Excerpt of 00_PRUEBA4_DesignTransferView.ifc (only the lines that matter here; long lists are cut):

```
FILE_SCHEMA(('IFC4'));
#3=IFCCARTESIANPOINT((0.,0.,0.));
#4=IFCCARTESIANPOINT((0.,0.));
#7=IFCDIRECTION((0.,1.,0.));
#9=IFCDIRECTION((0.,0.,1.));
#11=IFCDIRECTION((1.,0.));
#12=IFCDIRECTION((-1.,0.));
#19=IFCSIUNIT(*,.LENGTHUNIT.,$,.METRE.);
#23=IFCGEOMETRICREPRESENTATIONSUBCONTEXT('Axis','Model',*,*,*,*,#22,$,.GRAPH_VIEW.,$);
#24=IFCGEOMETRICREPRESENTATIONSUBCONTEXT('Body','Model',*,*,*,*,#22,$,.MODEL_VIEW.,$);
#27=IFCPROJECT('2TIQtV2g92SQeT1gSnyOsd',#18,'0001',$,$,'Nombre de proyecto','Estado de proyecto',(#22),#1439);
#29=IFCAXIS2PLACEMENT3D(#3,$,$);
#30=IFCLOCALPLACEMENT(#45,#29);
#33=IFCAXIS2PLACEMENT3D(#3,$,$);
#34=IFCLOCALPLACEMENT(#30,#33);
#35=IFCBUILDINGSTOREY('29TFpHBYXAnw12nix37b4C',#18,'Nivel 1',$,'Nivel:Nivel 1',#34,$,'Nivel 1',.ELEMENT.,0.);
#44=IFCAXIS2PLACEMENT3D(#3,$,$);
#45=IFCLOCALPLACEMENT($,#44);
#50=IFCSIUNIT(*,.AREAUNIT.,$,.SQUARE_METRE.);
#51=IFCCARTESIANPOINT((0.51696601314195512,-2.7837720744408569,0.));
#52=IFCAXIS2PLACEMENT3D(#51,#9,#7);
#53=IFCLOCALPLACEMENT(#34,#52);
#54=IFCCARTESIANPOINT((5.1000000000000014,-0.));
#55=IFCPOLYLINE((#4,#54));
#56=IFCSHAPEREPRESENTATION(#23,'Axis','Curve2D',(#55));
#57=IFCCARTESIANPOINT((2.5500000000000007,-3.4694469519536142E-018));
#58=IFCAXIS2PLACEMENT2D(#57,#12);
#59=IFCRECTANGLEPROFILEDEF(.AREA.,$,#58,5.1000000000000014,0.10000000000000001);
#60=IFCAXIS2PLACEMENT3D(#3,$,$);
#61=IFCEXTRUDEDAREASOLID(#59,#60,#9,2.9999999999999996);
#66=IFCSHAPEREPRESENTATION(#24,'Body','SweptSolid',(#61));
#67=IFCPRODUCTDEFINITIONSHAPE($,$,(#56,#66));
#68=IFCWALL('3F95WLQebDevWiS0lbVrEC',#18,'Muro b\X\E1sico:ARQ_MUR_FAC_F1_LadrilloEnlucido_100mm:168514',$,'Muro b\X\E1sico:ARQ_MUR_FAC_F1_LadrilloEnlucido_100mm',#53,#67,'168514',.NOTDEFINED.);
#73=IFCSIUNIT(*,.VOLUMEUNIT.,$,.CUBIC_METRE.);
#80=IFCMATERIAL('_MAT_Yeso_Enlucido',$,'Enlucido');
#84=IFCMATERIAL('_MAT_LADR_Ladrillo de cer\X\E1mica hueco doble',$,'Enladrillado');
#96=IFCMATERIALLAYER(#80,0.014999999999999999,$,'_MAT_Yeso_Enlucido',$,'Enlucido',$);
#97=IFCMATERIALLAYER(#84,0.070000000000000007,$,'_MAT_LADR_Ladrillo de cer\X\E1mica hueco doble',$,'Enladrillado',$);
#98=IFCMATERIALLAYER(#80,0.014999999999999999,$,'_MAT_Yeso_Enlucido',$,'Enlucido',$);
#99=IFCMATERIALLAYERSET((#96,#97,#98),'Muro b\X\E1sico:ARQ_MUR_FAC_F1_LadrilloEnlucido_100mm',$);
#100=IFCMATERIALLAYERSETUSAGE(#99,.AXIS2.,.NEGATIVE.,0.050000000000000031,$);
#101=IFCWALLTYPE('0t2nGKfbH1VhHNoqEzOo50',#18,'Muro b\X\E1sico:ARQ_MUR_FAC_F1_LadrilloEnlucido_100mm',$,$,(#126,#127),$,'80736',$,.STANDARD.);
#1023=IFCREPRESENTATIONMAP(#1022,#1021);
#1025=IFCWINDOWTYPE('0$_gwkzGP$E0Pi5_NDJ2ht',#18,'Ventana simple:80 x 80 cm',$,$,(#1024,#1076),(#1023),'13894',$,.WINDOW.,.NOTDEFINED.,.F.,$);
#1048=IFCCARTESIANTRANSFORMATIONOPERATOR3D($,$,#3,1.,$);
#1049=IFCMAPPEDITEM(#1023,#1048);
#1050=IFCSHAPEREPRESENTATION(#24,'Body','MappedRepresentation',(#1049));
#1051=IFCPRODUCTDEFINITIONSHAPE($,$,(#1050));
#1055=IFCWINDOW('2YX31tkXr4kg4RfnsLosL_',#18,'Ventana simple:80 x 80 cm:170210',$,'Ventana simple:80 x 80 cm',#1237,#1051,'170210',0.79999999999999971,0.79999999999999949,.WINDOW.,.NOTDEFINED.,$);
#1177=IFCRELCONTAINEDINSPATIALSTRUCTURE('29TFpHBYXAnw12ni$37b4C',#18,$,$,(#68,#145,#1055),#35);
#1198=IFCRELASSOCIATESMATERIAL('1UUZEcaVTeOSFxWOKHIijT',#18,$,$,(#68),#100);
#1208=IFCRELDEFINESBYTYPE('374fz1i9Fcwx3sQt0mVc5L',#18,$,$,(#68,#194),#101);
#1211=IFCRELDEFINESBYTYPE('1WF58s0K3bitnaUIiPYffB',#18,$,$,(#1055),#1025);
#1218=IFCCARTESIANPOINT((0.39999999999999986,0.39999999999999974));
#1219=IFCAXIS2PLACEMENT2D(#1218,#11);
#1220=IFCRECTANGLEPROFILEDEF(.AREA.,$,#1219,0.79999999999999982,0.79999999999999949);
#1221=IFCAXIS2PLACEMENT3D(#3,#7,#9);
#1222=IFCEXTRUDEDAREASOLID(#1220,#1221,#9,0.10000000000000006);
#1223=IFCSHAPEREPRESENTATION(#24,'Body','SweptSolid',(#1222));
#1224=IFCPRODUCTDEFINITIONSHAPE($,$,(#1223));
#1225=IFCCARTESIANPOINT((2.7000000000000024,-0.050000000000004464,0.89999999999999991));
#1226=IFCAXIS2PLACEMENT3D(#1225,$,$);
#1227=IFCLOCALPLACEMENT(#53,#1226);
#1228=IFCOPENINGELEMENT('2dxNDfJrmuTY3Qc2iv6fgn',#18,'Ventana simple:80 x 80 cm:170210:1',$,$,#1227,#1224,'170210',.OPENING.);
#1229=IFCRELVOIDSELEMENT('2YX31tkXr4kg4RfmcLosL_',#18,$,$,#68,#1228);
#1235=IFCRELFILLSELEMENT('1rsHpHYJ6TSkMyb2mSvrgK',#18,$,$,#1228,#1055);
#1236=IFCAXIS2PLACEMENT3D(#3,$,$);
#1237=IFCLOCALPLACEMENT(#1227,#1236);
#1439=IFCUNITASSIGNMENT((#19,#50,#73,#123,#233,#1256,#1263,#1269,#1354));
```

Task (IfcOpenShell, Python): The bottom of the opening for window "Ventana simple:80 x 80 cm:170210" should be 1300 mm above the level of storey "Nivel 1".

```python
import numpy as np
import ifcopenshell
import ifcopenshell.api.geometry
import ifcopenshell.geom
import ifcopenshell.util.element
import ifcopenshell.util.placement
import ifcopenshell.util.shape
import ifcopenshell.util.unit

model = ifcopenshell.open("00_PRUEBA4_DesignTransferView.ifc")
unit_scale = ifcopenshell.util.unit.calculate_unit_scale(model)

window = model.by_guid("2YX31tkXr4kg4RfnsLosL_")
opening = window.FillsVoids[0].RelatingOpeningElement
storey = ifcopenshell.util.element.get_container(window, ifc_class="IfcBuildingStorey")
level = ifcopenshell.util.placement.get_local_placement(storey.ObjectPlacement)[2, 3]

# The opening's origin need not be at the sill, so measure its lowest point.
shape = ifcopenshell.geom.create_shape(ifcopenshell.geom.settings(), opening)
bottom = ifcopenshell.util.shape.get_shape_bottom_elevation(shape, shape.geometry) / unit_scale
dz = level + 1.3 - bottom

shift = np.array([0.0, 0.0, dz])
# The window is placed relative to its opening, so it follows when the opening moves.
matrix = ifcopenshell.util.placement.get_local_placement(opening.ObjectPlacement)
matrix[:3, 3] += shift
ifcopenshell.api.geometry.edit_object_placement(
    model, product=opening, matrix=matrix, is_si=False, should_transform_children=True
)

print(f"moved by {dz * unit_scale:+.3f} m")

model.write("00_PRUEBA4_DesignTransferView_updated.ifc")
```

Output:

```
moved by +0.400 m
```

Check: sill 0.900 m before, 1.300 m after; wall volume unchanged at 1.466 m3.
